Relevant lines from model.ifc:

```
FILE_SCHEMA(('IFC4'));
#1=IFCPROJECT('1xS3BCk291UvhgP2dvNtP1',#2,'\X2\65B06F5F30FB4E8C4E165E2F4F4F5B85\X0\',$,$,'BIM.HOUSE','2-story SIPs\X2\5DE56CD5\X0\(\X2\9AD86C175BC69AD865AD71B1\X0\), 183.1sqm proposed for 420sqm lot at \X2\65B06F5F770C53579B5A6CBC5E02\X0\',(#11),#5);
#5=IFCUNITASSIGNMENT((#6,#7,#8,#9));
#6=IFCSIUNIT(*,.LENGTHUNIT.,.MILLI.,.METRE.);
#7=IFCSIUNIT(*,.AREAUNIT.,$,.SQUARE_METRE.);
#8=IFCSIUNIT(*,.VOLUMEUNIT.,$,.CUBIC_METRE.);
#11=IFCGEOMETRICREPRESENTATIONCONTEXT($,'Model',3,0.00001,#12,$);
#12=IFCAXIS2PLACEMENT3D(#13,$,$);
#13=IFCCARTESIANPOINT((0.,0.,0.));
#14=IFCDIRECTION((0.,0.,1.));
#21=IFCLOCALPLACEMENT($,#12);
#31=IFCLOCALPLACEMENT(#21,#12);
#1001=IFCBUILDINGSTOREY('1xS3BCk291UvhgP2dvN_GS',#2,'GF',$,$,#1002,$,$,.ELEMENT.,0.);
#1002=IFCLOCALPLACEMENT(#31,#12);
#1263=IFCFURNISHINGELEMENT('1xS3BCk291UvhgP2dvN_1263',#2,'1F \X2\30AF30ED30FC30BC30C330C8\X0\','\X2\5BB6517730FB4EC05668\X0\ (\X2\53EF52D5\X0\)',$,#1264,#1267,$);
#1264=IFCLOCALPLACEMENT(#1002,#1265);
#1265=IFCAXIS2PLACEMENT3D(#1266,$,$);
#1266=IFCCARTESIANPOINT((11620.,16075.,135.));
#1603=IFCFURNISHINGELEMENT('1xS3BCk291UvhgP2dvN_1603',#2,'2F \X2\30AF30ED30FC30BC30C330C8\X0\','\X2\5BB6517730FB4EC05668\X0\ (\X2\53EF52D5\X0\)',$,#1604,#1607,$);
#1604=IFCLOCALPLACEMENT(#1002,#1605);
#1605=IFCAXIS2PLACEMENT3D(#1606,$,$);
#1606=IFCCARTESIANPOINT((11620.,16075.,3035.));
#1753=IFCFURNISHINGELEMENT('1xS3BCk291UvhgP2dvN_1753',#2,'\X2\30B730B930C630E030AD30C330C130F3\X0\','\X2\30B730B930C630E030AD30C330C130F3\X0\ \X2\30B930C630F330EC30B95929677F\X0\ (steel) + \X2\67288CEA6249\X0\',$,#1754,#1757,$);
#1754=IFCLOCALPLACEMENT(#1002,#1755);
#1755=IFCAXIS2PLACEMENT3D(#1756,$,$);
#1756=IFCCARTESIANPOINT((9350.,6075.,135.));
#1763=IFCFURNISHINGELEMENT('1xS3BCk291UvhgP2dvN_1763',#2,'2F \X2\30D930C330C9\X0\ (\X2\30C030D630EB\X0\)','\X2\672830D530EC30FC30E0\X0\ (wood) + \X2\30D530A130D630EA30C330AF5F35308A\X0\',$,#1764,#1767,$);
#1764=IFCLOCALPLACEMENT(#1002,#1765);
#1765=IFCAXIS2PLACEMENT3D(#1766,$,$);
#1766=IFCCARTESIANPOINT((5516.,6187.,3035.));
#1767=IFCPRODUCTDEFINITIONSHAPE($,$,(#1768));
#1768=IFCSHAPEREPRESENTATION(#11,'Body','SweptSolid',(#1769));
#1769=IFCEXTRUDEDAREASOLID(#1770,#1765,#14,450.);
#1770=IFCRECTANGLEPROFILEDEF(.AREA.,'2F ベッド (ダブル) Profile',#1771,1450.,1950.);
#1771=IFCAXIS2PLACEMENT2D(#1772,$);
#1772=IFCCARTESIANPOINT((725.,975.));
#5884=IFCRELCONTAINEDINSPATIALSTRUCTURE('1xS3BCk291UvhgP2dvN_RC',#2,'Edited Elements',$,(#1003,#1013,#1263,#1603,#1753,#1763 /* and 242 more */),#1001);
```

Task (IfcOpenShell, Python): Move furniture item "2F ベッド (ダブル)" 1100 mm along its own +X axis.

```python
import ifcopenshell
import ifcopenshell.api.geometry
import ifcopenshell.util.placement

model = ifcopenshell.open("model.ifc")

item = model.by_guid("1xS3BCk291UvhgP2dvN_1763")
matrix = ifcopenshell.util.placement.get_local_placement(item.ObjectPlacement)
matrix[:3, 3] += matrix[:3, 0] * 1100.0
ifcopenshell.api.geometry.edit_object_placement(model, product=item, matrix=matrix, is_si=False)

print(ifcopenshell.util.placement.get_local_placement(item.ObjectPlacement).round(3) + 0.0)

model.write("model-out.ifc")
```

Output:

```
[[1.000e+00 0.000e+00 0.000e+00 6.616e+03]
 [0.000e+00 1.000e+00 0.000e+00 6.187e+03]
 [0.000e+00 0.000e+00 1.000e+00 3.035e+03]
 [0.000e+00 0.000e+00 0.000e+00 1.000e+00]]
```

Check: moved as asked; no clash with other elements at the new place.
